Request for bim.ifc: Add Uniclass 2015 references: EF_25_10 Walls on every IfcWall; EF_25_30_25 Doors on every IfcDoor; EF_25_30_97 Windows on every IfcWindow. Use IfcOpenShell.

First a look at what the model holds.

```python
import ifcopenshell

model = ifcopenshell.open("bim.ifc")
print(model.schema)
print("classifications:", [c.Name for c in model.by_type("IfcClassification")])
for ifc_class in ("IfcDoor", "IfcRoof", "IfcStair", "IfcWall", "IfcWindow"):
    print(ifc_class, len(model.by_type(ifc_class)))
```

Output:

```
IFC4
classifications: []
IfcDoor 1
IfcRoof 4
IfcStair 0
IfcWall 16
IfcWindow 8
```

```python
import ifcopenshell
import ifcopenshell.api.classification

model = ifcopenshell.open("bim.ifc")

system = ifcopenshell.api.classification.add_classification(model, classification="Uniclass 2015")

codes = {
    "IfcWall": ("EF_25_10", "Walls"),
    "IfcDoor": ("EF_25_30_25", "Doors"),
    "IfcWindow": ("EF_25_30_97", "Windows"),
}
for ifc_class, (code, name) in codes.items():
    products = model.by_type(ifc_class)
    ifcopenshell.api.classification.add_reference(
        model, products=products, classification=system, identification=code, name=name
    )
    print(code, len(products))

model.write("bim_rev.ifc")
```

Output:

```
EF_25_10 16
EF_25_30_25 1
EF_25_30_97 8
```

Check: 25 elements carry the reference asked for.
